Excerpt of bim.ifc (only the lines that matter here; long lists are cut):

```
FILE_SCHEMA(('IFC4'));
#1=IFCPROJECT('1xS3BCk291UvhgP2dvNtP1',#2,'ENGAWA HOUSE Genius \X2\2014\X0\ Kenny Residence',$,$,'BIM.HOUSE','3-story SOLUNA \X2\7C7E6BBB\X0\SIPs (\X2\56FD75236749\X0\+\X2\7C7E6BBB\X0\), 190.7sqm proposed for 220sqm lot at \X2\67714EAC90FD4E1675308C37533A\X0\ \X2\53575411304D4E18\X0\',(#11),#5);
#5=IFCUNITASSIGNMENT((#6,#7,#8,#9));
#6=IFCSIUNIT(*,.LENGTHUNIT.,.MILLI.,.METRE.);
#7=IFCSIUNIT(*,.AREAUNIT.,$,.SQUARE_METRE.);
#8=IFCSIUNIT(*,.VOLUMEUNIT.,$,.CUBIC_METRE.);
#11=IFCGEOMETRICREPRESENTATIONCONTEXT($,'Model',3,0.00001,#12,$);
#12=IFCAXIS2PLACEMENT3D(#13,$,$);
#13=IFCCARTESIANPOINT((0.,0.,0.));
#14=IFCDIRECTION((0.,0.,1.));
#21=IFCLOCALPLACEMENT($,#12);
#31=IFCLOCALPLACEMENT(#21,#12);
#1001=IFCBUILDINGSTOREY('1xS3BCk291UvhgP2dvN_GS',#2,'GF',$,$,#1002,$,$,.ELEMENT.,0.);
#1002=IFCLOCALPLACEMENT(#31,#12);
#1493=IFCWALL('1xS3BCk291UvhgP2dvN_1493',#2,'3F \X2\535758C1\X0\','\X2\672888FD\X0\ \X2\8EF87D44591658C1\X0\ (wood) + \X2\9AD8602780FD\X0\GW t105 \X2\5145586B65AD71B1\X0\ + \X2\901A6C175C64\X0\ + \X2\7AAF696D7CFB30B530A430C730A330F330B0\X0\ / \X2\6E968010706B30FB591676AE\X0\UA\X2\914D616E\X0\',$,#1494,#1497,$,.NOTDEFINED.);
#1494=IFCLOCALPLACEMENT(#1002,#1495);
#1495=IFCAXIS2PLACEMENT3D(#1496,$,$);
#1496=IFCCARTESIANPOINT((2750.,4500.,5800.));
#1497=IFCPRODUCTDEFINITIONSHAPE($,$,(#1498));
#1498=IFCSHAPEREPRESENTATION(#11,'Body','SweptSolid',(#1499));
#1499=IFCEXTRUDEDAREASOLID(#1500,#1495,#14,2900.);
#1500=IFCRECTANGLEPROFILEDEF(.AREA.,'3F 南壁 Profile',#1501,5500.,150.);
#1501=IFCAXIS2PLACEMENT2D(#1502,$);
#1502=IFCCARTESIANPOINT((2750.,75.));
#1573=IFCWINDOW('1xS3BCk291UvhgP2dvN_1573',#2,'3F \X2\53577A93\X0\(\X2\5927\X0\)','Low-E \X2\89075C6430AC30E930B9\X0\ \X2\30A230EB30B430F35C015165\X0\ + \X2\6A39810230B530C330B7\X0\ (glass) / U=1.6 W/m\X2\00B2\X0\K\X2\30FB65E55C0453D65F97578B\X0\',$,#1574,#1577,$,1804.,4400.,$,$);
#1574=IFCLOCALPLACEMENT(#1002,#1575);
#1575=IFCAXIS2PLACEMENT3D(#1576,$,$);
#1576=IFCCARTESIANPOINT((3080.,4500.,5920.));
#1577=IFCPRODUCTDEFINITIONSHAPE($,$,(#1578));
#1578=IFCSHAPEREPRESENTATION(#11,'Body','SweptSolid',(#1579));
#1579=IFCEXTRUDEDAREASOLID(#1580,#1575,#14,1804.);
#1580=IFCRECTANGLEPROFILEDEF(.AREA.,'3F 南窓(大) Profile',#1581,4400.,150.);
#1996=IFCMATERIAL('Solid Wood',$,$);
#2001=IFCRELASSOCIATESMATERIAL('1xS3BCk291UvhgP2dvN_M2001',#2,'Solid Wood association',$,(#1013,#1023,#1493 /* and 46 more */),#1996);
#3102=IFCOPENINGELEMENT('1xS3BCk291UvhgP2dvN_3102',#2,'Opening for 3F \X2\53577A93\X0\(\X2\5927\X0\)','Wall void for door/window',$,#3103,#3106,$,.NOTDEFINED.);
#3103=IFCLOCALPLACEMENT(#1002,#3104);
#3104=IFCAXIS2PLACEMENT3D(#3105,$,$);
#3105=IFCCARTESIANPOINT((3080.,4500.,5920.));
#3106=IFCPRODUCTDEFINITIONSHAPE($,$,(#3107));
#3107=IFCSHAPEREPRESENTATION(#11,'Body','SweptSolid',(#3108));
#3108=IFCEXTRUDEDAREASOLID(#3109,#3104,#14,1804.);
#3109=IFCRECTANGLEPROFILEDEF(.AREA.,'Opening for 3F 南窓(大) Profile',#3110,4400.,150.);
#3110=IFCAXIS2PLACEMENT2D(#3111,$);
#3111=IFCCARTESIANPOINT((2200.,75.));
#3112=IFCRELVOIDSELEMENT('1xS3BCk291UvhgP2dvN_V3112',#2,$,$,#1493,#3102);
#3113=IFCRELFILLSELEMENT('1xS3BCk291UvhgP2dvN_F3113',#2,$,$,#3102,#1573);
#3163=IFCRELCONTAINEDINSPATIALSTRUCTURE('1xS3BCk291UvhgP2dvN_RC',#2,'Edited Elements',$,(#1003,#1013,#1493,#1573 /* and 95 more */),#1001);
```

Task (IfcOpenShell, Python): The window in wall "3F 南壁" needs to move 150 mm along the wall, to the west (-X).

```python
import ifcopenshell
import ifcopenshell.api.geometry
import ifcopenshell.util.placement

model = ifcopenshell.open("bim.ifc")

window = model.by_guid("1xS3BCk291UvhgP2dvN_1573")
opening = window.FillsVoids[0].RelatingOpeningElement
wall = opening.VoidsElements[0].RelatingBuildingElement

wall_matrix = ifcopenshell.util.placement.get_local_placement(wall.ObjectPlacement)
shift = wall_matrix[:3, 0] * -150.0
before = ifcopenshell.util.placement.get_local_placement(window.ObjectPlacement)[:3, 3].copy()

# The window is not placed relative to its opening, so move both.
for product in (opening, window):
    matrix = ifcopenshell.util.placement.get_local_placement(product.ObjectPlacement)
    matrix[:3, 3] += shift
    ifcopenshell.api.geometry.edit_object_placement(model, product=product, matrix=matrix, is_si=False)

after = ifcopenshell.util.placement.get_local_placement(window.ObjectPlacement)[:3, 3]
print("window moved by", (after - before).round(3) + 0.0)

model.write("bim-out.ifc")
```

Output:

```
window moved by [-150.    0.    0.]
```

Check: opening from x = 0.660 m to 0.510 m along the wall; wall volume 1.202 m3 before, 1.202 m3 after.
